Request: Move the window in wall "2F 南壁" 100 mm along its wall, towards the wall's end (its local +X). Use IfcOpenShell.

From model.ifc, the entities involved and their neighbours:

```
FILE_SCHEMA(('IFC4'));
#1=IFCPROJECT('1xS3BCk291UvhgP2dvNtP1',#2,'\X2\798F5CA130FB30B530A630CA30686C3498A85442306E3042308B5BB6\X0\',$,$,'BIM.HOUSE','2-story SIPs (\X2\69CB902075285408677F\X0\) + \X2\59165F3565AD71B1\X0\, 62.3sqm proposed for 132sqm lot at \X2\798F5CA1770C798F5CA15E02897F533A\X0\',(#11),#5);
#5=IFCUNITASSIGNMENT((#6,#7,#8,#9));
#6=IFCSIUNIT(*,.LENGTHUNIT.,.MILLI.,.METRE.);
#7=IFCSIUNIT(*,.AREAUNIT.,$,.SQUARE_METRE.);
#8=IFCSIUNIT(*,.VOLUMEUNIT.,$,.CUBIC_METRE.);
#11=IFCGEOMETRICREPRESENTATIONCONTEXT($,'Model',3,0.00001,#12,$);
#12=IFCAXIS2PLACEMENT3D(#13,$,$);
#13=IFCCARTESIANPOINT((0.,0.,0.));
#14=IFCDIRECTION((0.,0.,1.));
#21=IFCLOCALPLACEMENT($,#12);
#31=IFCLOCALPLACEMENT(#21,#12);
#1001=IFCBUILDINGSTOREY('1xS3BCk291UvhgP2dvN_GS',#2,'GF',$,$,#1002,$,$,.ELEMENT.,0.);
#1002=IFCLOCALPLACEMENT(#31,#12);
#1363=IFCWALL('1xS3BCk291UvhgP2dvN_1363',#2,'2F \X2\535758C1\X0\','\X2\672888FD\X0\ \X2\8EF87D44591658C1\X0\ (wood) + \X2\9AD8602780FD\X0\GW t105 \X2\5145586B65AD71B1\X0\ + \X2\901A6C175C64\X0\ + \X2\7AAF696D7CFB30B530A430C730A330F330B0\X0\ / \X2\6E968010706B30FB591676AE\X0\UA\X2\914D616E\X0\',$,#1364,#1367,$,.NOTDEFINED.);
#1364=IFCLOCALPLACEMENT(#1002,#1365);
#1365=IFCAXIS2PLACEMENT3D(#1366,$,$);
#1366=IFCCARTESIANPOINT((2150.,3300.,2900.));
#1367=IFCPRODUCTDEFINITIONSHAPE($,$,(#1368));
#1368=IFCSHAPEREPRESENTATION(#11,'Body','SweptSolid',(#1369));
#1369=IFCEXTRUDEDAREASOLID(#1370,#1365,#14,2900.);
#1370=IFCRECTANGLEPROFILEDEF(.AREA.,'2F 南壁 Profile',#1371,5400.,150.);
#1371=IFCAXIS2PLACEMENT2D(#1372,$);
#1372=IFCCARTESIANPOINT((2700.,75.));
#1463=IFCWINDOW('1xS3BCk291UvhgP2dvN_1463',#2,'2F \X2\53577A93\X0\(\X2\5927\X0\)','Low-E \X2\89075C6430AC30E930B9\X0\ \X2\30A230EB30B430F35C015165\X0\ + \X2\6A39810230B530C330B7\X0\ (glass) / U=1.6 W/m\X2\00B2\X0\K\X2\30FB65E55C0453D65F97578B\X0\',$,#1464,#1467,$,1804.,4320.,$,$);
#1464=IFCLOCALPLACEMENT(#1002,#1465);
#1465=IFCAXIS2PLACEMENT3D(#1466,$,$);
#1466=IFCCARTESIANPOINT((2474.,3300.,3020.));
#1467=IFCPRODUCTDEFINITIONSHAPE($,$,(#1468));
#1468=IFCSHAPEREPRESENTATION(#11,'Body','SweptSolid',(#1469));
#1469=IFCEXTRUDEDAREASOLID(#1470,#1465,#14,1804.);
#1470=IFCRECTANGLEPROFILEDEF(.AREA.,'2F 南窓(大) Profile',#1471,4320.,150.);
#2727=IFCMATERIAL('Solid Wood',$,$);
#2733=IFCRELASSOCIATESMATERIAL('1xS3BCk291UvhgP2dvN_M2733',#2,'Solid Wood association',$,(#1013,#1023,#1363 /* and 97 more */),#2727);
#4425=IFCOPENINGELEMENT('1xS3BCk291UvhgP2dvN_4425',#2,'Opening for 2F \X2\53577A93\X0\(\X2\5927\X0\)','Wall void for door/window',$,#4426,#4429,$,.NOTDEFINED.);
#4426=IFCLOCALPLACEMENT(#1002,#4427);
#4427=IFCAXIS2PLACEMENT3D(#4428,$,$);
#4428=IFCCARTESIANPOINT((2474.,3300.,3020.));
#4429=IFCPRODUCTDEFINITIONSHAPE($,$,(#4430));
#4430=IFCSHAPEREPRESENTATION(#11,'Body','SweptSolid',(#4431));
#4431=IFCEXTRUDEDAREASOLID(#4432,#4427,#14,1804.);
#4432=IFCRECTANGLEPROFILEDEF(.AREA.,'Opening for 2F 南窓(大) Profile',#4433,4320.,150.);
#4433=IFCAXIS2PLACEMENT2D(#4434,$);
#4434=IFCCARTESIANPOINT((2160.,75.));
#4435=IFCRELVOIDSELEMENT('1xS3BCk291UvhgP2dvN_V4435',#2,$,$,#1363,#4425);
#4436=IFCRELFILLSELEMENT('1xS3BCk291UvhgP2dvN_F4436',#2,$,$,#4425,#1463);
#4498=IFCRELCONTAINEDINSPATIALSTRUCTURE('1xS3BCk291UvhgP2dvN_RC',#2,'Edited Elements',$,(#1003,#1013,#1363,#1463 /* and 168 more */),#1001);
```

```python
import ifcopenshell
import ifcopenshell.api.geometry
import ifcopenshell.util.placement
import ifcopenshell.util.unit

model = ifcopenshell.open("model.ifc")
unit_scale = ifcopenshell.util.unit.calculate_unit_scale(model)

window = model.by_guid("1xS3BCk291UvhgP2dvN_1463")
opening = window.FillsVoids[0].RelatingOpeningElement
wall = opening.VoidsElements[0].RelatingBuildingElement

wall_matrix = ifcopenshell.util.placement.get_local_placement(wall.ObjectPlacement)
shift = wall_matrix[:3, 0] * 0.1 / unit_scale
before = ifcopenshell.util.placement.get_local_placement(window.ObjectPlacement)[:3, 3].copy()

# The window is not placed relative to its opening, so move both.
for product in (opening, window):
    matrix = ifcopenshell.util.placement.get_local_placement(product.ObjectPlacement)
    matrix[:3, 3] += shift
    ifcopenshell.api.geometry.edit_object_placement(model, product=product, matrix=matrix, is_si=False)

after = ifcopenshell.util.placement.get_local_placement(window.ObjectPlacement)[:3, 3]
print("window moved by", (after - before).round(3) + 0.0)

model.write("model-out.ifc")
```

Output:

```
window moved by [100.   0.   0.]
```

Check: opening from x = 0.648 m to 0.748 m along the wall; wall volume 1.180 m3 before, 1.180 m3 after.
